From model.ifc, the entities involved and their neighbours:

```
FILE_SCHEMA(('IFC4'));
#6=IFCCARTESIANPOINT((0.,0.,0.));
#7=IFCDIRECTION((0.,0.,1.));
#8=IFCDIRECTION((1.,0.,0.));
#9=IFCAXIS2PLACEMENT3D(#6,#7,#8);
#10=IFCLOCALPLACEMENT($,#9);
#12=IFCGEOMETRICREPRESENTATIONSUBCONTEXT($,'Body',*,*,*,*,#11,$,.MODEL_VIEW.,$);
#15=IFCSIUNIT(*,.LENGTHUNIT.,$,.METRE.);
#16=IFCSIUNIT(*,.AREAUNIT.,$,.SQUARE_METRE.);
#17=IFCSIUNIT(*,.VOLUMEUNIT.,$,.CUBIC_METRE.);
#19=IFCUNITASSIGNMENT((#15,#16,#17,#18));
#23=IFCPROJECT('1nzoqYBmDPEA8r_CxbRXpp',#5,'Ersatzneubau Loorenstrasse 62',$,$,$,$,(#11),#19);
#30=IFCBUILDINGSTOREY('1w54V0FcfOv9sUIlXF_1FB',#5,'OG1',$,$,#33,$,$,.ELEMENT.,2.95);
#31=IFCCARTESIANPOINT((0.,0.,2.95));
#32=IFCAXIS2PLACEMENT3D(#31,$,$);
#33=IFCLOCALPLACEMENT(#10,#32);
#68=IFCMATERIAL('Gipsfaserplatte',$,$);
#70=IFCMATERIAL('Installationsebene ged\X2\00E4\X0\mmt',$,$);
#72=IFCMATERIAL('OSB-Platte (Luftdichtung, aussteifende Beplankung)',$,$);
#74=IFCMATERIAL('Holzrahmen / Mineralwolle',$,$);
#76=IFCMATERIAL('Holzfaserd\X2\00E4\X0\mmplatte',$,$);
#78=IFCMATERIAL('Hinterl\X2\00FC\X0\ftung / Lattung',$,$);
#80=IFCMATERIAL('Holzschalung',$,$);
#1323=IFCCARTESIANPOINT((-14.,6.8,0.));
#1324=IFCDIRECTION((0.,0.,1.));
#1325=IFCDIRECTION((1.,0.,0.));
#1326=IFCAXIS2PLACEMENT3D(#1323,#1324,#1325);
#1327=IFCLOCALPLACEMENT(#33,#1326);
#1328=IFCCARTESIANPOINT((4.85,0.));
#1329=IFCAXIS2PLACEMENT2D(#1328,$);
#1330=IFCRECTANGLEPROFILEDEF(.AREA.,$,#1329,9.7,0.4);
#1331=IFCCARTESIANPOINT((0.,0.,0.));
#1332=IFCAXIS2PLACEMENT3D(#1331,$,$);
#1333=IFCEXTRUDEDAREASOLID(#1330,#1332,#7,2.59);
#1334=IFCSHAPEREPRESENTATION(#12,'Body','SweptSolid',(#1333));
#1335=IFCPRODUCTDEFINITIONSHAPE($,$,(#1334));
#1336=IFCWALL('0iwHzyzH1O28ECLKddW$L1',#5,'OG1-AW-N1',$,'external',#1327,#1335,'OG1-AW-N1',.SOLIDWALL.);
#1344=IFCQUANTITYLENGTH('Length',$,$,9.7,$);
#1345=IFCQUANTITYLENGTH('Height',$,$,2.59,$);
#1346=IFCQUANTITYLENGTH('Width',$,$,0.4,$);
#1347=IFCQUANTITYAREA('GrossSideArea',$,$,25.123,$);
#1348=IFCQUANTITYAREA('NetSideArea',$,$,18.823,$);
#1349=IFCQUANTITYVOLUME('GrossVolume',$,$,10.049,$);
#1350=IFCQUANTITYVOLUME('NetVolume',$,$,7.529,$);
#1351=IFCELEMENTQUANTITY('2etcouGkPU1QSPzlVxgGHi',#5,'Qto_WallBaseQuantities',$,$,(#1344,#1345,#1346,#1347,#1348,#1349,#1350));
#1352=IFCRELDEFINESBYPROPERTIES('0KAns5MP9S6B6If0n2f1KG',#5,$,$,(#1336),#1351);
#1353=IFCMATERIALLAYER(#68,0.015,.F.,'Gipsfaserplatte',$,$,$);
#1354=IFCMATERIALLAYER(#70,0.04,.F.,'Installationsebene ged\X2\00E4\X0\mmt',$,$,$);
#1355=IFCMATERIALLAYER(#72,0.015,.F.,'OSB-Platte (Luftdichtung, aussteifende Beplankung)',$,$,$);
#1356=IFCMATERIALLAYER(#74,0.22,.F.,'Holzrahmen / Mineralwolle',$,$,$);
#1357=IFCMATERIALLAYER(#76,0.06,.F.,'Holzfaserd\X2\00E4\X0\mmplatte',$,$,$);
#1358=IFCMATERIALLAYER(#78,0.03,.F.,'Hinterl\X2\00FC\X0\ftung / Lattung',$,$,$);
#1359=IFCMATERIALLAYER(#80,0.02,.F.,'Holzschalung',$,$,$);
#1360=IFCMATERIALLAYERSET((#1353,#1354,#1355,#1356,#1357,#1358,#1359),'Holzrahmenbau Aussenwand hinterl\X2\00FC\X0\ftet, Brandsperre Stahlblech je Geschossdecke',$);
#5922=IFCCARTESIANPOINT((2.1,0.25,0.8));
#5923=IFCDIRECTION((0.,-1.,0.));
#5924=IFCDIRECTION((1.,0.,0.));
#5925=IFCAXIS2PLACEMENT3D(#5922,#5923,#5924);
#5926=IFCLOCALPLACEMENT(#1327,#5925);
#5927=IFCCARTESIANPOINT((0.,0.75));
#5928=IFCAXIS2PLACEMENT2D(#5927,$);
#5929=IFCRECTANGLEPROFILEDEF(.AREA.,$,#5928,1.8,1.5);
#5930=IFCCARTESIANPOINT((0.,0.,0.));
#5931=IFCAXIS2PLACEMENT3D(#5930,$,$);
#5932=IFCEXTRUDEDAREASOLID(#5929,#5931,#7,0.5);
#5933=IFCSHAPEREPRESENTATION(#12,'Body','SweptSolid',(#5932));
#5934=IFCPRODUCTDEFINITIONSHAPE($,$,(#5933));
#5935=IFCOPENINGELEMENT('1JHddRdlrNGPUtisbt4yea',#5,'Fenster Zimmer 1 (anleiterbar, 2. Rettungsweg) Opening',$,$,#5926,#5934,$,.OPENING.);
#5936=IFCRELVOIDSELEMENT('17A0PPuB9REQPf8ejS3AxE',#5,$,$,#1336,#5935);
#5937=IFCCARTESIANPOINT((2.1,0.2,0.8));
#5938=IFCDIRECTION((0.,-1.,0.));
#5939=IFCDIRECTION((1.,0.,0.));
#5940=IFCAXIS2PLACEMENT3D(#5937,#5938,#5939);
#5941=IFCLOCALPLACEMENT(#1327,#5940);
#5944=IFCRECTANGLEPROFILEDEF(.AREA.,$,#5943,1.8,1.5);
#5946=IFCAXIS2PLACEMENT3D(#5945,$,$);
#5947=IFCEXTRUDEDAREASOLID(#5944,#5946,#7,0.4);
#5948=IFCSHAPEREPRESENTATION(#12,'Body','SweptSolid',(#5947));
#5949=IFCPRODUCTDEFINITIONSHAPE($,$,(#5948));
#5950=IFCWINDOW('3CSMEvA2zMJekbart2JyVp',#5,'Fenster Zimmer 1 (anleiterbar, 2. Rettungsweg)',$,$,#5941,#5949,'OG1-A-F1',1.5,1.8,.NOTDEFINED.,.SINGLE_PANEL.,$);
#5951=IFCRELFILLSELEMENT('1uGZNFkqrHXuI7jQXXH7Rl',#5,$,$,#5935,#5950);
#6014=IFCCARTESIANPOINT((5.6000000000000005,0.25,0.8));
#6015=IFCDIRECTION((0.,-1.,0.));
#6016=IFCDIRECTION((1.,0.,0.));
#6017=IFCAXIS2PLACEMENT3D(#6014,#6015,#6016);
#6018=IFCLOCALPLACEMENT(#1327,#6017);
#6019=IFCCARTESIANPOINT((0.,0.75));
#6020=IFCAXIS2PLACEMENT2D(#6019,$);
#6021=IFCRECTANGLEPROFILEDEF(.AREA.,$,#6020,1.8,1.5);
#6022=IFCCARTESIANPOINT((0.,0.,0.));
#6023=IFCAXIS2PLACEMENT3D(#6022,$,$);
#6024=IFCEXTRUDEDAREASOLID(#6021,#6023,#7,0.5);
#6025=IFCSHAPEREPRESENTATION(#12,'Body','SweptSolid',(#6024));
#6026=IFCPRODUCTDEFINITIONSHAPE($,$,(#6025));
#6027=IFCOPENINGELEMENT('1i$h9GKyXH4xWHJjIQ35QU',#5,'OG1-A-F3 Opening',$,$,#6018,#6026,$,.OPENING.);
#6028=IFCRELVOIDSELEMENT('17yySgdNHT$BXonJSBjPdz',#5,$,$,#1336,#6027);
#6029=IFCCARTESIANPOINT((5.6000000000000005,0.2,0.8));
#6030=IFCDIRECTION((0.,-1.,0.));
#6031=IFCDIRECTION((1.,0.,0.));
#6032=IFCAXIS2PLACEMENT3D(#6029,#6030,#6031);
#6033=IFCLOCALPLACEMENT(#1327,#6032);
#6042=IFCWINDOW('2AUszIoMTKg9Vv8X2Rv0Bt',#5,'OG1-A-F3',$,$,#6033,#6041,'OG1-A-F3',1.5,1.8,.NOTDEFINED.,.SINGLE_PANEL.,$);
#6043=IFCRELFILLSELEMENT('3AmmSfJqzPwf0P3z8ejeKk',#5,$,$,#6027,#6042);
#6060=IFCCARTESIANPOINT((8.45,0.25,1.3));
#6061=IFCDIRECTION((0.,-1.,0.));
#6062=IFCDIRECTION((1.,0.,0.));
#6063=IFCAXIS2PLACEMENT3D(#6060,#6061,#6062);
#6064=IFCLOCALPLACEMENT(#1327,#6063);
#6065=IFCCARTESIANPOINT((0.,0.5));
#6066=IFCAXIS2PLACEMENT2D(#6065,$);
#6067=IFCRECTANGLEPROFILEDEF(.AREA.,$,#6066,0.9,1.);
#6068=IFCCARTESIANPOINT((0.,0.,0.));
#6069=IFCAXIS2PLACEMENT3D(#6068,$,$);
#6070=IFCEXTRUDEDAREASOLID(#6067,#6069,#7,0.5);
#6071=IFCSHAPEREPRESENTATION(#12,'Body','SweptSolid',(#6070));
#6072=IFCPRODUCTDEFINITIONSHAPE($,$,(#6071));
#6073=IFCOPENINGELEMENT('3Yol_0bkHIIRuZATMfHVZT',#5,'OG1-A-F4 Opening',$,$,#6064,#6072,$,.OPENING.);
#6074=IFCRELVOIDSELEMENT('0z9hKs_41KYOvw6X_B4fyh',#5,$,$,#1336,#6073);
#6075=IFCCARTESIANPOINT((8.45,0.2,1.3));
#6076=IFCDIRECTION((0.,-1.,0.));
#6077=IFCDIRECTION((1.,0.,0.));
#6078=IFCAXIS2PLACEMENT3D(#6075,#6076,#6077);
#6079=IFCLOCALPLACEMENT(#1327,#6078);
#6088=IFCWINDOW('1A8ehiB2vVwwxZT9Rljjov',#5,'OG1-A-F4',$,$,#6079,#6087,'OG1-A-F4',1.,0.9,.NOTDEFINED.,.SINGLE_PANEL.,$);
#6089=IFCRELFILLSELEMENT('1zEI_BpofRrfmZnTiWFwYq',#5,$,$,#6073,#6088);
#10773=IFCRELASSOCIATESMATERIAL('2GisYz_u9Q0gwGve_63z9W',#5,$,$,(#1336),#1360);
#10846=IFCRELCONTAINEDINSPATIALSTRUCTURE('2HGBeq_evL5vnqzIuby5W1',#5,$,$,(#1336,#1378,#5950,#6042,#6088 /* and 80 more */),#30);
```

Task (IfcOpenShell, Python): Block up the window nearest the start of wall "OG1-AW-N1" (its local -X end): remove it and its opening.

```python
import ifcopenshell
import ifcopenshell.api.feature
import ifcopenshell.api.pset
import ifcopenshell.api.root
import ifcopenshell.geom
import ifcopenshell.util.element
import ifcopenshell.util.shape
import ifcopenshell.util.unit

model = ifcopenshell.open("model.ifc")
area_scale = ifcopenshell.util.unit.calculate_unit_scale(model, "AREAUNIT")
volume_scale = ifcopenshell.util.unit.calculate_unit_scale(model, "VOLUMEUNIT")
settings = ifcopenshell.geom.settings()


def volume(element):
    """Net volume in cubic metres, openings subtracted."""
    shape = ifcopenshell.geom.create_shape(settings, element)
    return ifcopenshell.util.shape.get_volume(shape.geometry)


window = model.by_id(5950)
opening = window.FillsVoids[0].RelatingOpeningElement
wall = opening.VoidsElements[0].RelatingBuildingElement
before = volume(wall)

ifcopenshell.api.root.remove_product(model, product=window)
ifcopenshell.api.feature.remove_feature(model, feature=opening)

after = volume(wall)
thickness = 0.4  # wall thickness in metres

# Update the wall's stored quantities.
qto = model.by_id(ifcopenshell.util.element.get_pset(wall, "Qto_WallBaseQuantities", should_inherit=False)["id"])
ifcopenshell.api.pset.edit_qto(model, qto=qto, properties={
    "NetSideArea": after / thickness / area_scale,
    "NetVolume": after / volume_scale,
})

print(f"wall volume {before:.3f} -> {after:.3f} m3")

model.write("model_v2.ifc")
```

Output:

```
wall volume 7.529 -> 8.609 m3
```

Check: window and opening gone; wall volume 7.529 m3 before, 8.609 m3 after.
